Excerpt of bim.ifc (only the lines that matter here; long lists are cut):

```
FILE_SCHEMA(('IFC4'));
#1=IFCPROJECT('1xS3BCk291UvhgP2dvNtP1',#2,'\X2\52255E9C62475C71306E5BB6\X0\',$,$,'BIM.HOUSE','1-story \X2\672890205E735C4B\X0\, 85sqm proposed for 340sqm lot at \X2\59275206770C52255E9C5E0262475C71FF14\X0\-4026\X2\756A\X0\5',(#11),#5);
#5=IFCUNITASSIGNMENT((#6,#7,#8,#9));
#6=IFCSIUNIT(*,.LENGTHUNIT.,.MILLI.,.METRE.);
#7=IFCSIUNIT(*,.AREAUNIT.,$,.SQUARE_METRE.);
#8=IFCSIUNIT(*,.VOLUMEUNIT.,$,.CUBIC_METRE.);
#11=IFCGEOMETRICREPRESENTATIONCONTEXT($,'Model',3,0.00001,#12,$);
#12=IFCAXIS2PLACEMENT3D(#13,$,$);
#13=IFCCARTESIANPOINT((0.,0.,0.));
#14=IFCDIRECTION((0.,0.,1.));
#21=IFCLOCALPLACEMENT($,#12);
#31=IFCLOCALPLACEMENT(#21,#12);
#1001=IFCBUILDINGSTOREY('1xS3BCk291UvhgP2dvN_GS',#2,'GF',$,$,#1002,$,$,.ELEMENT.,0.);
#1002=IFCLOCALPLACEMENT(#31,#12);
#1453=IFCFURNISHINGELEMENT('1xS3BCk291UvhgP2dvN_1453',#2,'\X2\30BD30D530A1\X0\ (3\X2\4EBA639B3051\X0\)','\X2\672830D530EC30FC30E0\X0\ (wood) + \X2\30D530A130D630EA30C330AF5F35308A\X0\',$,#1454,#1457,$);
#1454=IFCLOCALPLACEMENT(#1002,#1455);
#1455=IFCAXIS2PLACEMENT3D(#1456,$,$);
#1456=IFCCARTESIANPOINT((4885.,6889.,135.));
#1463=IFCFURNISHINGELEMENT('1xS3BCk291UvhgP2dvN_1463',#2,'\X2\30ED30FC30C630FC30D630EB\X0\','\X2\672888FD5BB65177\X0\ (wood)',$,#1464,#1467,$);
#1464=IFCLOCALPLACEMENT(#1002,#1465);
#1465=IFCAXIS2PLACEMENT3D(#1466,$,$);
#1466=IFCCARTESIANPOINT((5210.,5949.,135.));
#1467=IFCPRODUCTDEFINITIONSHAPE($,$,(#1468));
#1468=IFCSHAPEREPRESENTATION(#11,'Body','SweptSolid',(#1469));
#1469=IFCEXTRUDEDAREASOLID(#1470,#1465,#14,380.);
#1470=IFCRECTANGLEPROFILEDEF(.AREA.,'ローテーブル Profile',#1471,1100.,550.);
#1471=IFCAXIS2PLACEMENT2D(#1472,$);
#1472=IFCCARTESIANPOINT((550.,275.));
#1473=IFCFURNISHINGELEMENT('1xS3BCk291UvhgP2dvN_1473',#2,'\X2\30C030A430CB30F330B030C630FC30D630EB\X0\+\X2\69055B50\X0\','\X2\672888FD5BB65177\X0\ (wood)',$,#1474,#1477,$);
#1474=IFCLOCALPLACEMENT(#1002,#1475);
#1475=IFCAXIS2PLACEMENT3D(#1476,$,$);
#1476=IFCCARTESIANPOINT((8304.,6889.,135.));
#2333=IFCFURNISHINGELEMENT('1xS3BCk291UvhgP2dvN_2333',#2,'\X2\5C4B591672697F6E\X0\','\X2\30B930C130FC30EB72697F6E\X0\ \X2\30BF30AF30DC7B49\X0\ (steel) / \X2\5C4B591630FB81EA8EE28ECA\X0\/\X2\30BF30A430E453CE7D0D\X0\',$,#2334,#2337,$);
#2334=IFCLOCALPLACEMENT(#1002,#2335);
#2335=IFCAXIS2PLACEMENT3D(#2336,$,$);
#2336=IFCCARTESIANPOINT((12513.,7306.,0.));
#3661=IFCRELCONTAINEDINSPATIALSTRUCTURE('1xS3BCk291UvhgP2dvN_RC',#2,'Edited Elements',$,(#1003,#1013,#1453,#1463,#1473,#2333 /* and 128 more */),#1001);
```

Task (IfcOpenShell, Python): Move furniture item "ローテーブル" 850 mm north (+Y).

```python
import ifcopenshell
import ifcopenshell.api.geometry
import ifcopenshell.util.placement

model = ifcopenshell.open("bim.ifc")

item = model.by_guid("1xS3BCk291UvhgP2dvN_1463")
matrix = ifcopenshell.util.placement.get_local_placement(item.ObjectPlacement)
matrix[1, 3] += 850.0
ifcopenshell.api.geometry.edit_object_placement(model, product=item, matrix=matrix, is_si=False)

print(ifcopenshell.util.placement.get_local_placement(item.ObjectPlacement).round(3) + 0.0)

model.write("bim_updated.ifc")
```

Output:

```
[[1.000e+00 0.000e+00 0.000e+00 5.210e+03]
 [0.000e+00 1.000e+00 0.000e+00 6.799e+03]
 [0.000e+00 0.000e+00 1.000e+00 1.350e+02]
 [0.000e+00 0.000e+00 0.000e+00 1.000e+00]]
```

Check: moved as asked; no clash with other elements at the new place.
